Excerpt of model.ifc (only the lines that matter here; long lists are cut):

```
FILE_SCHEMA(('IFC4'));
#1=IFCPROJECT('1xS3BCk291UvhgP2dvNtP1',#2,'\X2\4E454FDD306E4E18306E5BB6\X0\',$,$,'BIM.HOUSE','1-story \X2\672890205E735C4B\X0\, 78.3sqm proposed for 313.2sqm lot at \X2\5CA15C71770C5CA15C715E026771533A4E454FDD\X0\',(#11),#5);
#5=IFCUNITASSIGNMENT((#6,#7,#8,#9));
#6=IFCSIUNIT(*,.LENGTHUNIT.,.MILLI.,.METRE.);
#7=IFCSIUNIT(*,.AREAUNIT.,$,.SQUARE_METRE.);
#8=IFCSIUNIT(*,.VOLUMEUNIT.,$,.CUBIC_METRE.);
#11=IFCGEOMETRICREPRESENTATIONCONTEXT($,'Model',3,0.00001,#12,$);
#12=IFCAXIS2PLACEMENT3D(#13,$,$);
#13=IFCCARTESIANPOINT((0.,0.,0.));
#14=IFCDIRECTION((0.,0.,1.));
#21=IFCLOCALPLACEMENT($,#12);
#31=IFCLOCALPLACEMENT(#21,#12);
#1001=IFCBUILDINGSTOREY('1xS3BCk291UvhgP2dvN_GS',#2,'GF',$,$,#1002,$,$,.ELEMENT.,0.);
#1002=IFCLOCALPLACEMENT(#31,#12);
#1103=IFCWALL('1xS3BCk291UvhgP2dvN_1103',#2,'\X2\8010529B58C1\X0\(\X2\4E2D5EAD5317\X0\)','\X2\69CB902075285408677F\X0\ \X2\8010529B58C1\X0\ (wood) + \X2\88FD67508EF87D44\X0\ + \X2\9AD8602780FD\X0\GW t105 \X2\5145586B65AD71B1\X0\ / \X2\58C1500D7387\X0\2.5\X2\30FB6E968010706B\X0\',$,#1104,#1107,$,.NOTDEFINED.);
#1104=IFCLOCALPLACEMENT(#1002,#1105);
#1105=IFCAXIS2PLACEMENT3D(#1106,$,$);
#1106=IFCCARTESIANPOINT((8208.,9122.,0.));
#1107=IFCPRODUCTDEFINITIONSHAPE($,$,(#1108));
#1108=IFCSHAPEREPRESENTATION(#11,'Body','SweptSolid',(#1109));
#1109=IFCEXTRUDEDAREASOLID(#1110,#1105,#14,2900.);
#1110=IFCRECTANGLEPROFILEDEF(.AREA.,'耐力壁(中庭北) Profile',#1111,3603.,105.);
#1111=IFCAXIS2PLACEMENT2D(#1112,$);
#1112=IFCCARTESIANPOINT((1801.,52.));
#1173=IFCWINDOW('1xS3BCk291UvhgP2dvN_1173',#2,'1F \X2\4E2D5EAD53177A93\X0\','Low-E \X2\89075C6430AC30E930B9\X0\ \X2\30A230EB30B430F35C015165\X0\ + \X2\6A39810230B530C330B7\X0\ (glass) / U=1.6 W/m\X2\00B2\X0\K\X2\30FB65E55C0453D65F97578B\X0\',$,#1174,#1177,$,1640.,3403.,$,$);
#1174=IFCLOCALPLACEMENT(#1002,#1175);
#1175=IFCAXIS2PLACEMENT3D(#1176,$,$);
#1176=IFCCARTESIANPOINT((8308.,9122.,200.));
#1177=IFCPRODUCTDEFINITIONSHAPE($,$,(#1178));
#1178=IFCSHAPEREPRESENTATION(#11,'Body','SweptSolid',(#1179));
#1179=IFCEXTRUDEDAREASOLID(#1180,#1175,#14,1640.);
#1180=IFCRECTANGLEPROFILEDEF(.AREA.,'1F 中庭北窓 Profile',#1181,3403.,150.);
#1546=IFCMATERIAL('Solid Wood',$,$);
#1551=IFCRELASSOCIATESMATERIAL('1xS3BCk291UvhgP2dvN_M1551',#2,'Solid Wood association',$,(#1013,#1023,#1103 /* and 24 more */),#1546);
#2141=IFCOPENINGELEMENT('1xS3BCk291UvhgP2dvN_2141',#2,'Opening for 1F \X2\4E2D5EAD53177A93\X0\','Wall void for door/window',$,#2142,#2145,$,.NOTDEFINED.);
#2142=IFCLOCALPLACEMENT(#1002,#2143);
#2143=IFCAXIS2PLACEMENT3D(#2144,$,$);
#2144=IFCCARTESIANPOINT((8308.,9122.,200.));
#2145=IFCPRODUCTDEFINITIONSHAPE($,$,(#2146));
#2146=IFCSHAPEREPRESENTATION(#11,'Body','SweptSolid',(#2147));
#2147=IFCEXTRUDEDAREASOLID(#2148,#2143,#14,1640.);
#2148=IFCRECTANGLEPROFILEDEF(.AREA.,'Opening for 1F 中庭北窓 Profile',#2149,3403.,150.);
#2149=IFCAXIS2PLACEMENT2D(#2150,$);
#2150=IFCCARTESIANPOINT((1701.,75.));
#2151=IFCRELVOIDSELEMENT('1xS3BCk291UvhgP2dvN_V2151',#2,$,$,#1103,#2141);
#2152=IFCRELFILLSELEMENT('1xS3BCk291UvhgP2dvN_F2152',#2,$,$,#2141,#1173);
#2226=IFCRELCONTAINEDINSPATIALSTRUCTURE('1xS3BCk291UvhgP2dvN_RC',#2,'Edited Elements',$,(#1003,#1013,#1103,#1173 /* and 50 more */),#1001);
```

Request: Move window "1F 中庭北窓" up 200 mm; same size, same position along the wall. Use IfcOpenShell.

```python
import numpy as np
import ifcopenshell
import ifcopenshell.api.geometry
import ifcopenshell.util.placement
import ifcopenshell.util.unit

model = ifcopenshell.open("model.ifc")
unit_scale = ifcopenshell.util.unit.calculate_unit_scale(model)

window = model.by_id(1173)
opening = window.FillsVoids[0].RelatingOpeningElement
dz = 0.2 / unit_scale

shift = np.array([0.0, 0.0, dz])
# The window is not placed relative to its opening, so move both.
for product in (opening, window):
    matrix = ifcopenshell.util.placement.get_local_placement(product.ObjectPlacement)
    matrix[:3, 3] += shift
    ifcopenshell.api.geometry.edit_object_placement(model, product=product, matrix=matrix, is_si=False)

print(f"moved by {dz * unit_scale:+.3f} m")

model.write("model_v2.ifc")
```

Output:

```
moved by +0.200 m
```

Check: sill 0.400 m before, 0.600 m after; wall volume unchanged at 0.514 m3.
